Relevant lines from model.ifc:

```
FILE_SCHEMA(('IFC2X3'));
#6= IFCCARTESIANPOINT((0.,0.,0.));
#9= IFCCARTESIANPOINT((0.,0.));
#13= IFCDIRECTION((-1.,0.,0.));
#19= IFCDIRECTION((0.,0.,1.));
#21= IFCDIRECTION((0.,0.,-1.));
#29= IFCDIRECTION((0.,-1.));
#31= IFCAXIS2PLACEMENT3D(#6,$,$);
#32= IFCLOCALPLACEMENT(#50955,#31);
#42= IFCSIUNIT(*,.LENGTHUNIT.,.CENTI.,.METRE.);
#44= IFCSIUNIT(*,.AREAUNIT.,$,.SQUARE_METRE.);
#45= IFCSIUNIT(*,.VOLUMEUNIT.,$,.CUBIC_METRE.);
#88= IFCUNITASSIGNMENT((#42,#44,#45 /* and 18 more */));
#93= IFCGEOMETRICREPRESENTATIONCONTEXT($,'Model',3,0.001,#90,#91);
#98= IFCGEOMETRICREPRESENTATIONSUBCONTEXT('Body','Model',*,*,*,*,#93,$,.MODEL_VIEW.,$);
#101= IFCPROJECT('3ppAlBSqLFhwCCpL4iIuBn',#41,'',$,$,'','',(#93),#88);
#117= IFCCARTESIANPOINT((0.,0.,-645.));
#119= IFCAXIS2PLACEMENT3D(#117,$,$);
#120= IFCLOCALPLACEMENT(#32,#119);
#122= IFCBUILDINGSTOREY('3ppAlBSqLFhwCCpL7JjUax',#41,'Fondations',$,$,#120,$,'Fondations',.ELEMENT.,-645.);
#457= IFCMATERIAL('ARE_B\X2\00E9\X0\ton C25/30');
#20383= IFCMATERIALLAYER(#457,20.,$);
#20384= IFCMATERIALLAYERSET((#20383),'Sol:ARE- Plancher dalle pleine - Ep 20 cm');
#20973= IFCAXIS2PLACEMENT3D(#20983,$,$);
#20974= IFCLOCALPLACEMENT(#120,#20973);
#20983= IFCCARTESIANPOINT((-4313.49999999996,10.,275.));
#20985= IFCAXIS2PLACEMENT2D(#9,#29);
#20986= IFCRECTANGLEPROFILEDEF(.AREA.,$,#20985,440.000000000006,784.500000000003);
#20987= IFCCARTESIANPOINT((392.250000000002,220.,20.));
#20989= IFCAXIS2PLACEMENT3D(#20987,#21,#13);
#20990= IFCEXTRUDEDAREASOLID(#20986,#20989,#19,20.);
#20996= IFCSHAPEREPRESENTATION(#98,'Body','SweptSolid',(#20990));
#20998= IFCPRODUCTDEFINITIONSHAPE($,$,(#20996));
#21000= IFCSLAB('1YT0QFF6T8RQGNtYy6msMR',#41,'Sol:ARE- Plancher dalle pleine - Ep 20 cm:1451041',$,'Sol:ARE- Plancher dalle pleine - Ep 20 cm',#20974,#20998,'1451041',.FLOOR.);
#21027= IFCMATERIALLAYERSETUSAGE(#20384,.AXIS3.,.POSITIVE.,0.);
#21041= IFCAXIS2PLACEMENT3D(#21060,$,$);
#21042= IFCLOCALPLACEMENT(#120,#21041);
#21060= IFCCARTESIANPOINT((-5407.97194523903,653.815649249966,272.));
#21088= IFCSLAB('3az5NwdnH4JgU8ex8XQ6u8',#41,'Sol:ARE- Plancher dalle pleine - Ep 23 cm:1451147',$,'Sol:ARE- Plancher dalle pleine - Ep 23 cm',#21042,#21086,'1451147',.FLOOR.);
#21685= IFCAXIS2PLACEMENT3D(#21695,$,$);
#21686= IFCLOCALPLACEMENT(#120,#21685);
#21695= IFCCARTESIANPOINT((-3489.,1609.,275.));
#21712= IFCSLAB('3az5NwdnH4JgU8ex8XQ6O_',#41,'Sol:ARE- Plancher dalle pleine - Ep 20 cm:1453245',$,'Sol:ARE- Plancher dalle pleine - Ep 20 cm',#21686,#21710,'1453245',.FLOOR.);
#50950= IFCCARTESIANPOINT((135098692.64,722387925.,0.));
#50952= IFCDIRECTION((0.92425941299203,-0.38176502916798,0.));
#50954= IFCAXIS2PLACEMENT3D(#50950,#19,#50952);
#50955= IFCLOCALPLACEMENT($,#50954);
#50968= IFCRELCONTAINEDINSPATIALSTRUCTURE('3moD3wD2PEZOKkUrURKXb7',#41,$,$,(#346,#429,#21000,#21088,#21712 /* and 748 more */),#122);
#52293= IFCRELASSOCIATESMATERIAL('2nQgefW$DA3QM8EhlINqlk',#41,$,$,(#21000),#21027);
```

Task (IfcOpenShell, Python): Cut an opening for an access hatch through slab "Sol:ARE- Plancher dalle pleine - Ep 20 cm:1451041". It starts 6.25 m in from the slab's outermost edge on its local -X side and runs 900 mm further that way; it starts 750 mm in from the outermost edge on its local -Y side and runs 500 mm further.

```python
import numpy as np
import ifcopenshell
import ifcopenshell.api.feature
import ifcopenshell.api.geometry
import ifcopenshell.api.root
import ifcopenshell.geom
import ifcopenshell.util.placement
import ifcopenshell.util.representation
import ifcopenshell.util.shape
import ifcopenshell.util.unit

model = ifcopenshell.open("model.ifc")
unit_scale = ifcopenshell.util.unit.calculate_unit_scale(model)
settings = ifcopenshell.geom.settings()


def volume(element):
    """Net volume in cubic metres, openings subtracted."""
    shape = ifcopenshell.geom.create_shape(settings, element)
    return ifcopenshell.util.shape.get_volume(shape.geometry)


slab = model.by_id(21000)
before = volume(slab)

# Extent in the slab's own axes, in metres. The edges named are its -X and -Y sides.
slab_shape = ifcopenshell.geom.create_shape(settings, slab)
vertices = ifcopenshell.util.shape.get_vertices(slab_shape.geometry)
x_min, y_min, bottom = vertices.min(axis=0)
top = vertices[:, 2].max()

opening = ifcopenshell.api.root.create_entity(model, ifc_class="IfcOpeningElement", name="Access hatch opening")
context = ifcopenshell.util.representation.get_context(model, "Model", "Body", "MODEL_VIEW")
width, depth = 0.9, 0.5
outline = [(0.0, 0.0), (width, 0.0), (width, depth), (0.0, depth), (0.0, 0.0)]
# Overshoot both faces by 50 mm so the cut is clean.
shape = ifcopenshell.api.geometry.add_slab_representation(
    model, context=context, depth=top - bottom + 0.1, polyline=outline
)
ifcopenshell.api.geometry.assign_representation(model, product=opening, representation=shape)

matrix = ifcopenshell.util.placement.get_local_placement(slab.ObjectPlacement)
matrix[:, 3] = matrix @ np.append(np.array([x_min + 6.25, y_min + 0.75, bottom - 0.05]) / unit_scale, 1.0)
ifcopenshell.api.geometry.edit_object_placement(model, product=opening, matrix=matrix, is_si=False)
ifcopenshell.api.feature.add_feature(model, feature=opening, element=slab)

after = volume(slab)

print(f"slab volume {before:.3f} -> {after:.3f} m3")

model.write("model_v2.ifc")
```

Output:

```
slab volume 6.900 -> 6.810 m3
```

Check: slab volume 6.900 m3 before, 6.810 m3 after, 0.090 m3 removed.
